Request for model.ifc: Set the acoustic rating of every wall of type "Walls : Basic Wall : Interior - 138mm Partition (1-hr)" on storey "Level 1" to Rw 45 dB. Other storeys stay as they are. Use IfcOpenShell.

First a look at what the model holds.

```python
import ifcopenshell
import ifcopenshell.util.element

model = ifcopenshell.open("model.ifc")
print(model.schema)
storey = next(s for s in model.by_type("IfcBuildingStorey") if s.Name == "Level 1")
walls = [e for e in ifcopenshell.util.element.get_decomposition(storey) if e.is_a("IfcWall")]
seen = {}
for e in walls:
    element_type = ifcopenshell.util.element.get_type(e)
    key = (element_type.Name if element_type != e and element_type else None, ifcopenshell.util.element.get_pset(e, "Pset_WallCommon", "AcousticRating"))
    seen[key] = seen.get(key, 0) + 1
for (name, value), count in sorted(seen.items(), key=str):
    print(count, "x", name, "|", value)
```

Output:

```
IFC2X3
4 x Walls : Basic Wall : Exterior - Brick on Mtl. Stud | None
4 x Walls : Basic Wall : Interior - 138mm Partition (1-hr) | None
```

```python
import ifcopenshell
import ifcopenshell.api.pset
import ifcopenshell.util.element

model = ifcopenshell.open("model.ifc")

storey = next(s for s in model.by_type("IfcBuildingStorey") if s.Name == "Level 1")
walls = [e for e in ifcopenshell.util.element.get_decomposition(storey) if e.is_a("IfcWall")]

count = 0
for e in walls:
    element_type = ifcopenshell.util.element.get_type(e)
    if element_type in (None, e) or element_type.Name != "Walls : Basic Wall : Interior - 138mm Partition (1-hr)":
        continue
    # add_pset returns the element's existing set when there is one.
    pset = ifcopenshell.api.pset.add_pset(model, product=e, name="Pset_WallCommon")
    ifcopenshell.api.pset.edit_pset(model, pset=pset, properties={"AcousticRating": "Rw 45 dB"})
    count += 1

print(count, "walls updated")

model.write("model_edited.ifc")
```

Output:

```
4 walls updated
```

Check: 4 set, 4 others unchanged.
